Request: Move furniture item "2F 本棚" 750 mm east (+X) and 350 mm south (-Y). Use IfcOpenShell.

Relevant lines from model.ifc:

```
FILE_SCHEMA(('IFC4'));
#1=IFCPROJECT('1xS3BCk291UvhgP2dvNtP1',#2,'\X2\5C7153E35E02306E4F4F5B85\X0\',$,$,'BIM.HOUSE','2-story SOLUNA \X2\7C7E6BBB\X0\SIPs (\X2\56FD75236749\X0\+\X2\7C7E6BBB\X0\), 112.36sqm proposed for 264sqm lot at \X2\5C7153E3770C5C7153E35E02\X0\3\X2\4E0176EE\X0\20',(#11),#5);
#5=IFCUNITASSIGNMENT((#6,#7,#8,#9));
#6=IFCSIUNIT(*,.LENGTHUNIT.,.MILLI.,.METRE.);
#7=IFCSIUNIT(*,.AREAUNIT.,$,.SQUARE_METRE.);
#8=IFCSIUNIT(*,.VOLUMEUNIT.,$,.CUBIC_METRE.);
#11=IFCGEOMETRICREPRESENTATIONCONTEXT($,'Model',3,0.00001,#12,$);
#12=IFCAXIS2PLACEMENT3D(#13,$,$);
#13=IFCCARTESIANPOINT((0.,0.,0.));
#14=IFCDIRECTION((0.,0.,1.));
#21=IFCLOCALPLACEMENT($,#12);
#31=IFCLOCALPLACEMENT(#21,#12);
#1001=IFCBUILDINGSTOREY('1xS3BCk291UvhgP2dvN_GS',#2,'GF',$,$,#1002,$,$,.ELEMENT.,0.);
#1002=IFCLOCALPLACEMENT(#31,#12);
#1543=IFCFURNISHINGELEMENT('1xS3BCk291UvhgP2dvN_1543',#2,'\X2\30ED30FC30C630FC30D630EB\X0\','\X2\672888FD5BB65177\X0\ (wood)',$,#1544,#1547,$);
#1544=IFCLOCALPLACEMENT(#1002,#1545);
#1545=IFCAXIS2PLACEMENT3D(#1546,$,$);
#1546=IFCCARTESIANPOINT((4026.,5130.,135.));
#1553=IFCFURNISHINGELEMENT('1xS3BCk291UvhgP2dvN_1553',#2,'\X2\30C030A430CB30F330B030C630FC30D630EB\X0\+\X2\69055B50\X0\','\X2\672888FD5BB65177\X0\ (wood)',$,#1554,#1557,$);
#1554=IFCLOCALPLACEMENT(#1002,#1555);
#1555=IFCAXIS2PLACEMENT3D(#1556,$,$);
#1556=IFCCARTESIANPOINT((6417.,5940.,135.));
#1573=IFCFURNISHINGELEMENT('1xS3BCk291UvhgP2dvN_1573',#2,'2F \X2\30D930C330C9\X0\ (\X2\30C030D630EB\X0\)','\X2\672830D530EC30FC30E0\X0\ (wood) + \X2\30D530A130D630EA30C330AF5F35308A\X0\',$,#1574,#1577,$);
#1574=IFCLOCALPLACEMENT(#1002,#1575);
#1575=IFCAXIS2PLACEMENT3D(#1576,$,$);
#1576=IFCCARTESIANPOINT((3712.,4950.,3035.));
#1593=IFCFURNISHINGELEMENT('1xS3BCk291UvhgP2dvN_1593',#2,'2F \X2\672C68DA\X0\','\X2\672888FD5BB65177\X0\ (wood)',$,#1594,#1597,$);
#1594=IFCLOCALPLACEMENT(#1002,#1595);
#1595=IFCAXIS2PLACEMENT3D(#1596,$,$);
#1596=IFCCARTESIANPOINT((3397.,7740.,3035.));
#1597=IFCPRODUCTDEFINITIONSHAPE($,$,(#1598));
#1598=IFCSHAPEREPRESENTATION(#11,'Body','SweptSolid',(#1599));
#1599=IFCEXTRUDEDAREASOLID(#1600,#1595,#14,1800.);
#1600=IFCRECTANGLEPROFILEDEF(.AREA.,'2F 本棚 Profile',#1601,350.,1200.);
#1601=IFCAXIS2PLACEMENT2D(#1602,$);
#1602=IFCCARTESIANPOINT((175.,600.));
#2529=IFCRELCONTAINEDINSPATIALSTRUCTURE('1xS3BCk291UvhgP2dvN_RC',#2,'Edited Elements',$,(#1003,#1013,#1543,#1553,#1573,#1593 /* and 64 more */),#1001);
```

```python
import ifcopenshell
import ifcopenshell.api.geometry
import ifcopenshell.util.placement

model = ifcopenshell.open("model.ifc")

item = model.by_guid("1xS3BCk291UvhgP2dvN_1593")
matrix = ifcopenshell.util.placement.get_local_placement(item.ObjectPlacement)
matrix[0, 3] += 750.0
matrix[1, 3] -= 350.0
ifcopenshell.api.geometry.edit_object_placement(model, product=item, matrix=matrix, is_si=False)

print(ifcopenshell.util.placement.get_local_placement(item.ObjectPlacement).round(3) + 0.0)

model.write("model_v2.ifc")
```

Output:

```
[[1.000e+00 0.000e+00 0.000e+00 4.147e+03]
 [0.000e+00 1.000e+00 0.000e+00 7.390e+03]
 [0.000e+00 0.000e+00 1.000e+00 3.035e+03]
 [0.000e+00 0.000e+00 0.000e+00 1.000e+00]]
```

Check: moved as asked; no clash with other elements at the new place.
